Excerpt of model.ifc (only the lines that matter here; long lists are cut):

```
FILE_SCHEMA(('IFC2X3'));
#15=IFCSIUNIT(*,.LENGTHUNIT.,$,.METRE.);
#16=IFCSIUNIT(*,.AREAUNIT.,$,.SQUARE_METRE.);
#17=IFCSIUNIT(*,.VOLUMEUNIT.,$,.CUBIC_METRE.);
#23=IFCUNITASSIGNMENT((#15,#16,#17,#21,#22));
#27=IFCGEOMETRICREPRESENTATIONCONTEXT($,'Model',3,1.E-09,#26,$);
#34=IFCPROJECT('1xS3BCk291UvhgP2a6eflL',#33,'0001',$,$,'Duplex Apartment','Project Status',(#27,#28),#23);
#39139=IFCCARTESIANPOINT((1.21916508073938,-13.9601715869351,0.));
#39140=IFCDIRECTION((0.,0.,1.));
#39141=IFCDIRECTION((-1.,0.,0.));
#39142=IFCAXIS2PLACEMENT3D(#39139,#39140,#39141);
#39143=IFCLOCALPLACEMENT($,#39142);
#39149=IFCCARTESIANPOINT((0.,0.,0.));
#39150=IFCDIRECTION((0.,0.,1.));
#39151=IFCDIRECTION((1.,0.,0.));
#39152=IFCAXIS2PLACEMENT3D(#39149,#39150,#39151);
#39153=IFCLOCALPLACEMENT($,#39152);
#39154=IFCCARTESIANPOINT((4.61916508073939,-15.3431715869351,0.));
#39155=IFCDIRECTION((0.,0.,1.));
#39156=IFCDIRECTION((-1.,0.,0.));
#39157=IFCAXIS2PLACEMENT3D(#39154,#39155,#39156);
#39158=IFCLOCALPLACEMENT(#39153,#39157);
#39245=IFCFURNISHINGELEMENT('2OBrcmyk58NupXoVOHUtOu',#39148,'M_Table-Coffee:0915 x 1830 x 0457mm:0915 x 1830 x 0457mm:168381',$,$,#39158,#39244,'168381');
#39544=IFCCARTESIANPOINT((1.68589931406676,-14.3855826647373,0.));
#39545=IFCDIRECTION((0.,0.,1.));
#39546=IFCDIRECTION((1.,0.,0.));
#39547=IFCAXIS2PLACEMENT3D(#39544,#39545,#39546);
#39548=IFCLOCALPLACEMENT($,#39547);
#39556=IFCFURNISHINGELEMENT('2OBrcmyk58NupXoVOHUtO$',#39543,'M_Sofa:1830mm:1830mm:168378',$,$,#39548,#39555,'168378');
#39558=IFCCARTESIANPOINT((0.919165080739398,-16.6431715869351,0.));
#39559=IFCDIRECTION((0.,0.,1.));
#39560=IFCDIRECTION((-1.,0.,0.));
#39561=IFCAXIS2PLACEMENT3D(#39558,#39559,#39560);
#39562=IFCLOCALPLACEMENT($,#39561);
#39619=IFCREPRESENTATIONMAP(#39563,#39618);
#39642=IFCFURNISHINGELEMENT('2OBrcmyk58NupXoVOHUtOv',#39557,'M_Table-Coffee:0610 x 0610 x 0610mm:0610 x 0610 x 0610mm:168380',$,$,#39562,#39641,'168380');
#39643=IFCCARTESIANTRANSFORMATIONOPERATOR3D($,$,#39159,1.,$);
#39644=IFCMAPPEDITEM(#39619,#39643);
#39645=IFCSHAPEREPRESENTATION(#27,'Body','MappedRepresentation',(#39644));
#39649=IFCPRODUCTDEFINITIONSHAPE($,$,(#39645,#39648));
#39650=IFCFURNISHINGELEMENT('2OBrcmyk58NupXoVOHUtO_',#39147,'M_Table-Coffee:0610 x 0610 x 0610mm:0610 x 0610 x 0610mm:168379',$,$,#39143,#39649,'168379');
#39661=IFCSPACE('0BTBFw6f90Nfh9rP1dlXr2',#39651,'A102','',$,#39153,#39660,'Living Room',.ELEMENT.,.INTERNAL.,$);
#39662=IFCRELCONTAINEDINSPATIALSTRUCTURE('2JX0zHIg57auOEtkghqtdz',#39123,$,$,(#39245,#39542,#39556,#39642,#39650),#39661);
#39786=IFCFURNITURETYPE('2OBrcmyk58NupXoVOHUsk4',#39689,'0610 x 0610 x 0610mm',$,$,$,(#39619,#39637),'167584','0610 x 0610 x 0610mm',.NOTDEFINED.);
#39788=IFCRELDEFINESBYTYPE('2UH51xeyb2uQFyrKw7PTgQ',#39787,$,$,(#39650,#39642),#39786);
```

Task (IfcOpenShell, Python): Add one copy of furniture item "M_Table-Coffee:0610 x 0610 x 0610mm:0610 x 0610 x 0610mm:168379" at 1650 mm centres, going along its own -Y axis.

```python
import ifcopenshell
import ifcopenshell.api.geometry
import ifcopenshell.api.root
import ifcopenshell.util.element
import ifcopenshell.util.placement
import ifcopenshell.util.unit

model = ifcopenshell.open("model.ifc")
unit_scale = ifcopenshell.util.unit.calculate_unit_scale(model)


def reuse_history(source, copy):
    """copy_class also copies each property set's owner history, people and application; keep the originals."""
    for rel in copy.IsDefinedBy:
        if rel.is_a("IfcRelDefinesByProperties") and (history := rel.RelatingPropertyDefinition.OwnerHistory):
            rel.RelatingPropertyDefinition.OwnerHistory = source.OwnerHistory
            ifcopenshell.util.element.remove_deep2(model, history)


source = model.by_guid("2OBrcmyk58NupXoVOHUtO_")
base = ifcopenshell.util.placement.get_local_placement(source.ObjectPlacement)
step = -base[:3, 1] * 1.65 / unit_scale

for i in range(1, 2):
    copy = ifcopenshell.api.root.copy_class(model, product=source)
    copy.Representation = ifcopenshell.util.element.copy_deep(
        model, source.Representation, exclude=["IfcGeometricRepresentationContext", "IfcRepresentationMap"]
    )
    copy.Name = "M_Table-Coffee:0610 x 0610 x 0610mm:0610 x 0610 x 0610mm"
    copy.Tag = None
    reuse_history(source, copy)
    matrix = base.copy()
    matrix[:3, 3] += i * step
    print("added at", matrix[:3, 3].round(3) + 0.0)
    ifcopenshell.api.geometry.edit_object_placement(model, product=copy, matrix=matrix, is_si=False)

model.write("model_edited.ifc")
```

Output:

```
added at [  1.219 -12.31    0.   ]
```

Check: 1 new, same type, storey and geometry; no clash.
